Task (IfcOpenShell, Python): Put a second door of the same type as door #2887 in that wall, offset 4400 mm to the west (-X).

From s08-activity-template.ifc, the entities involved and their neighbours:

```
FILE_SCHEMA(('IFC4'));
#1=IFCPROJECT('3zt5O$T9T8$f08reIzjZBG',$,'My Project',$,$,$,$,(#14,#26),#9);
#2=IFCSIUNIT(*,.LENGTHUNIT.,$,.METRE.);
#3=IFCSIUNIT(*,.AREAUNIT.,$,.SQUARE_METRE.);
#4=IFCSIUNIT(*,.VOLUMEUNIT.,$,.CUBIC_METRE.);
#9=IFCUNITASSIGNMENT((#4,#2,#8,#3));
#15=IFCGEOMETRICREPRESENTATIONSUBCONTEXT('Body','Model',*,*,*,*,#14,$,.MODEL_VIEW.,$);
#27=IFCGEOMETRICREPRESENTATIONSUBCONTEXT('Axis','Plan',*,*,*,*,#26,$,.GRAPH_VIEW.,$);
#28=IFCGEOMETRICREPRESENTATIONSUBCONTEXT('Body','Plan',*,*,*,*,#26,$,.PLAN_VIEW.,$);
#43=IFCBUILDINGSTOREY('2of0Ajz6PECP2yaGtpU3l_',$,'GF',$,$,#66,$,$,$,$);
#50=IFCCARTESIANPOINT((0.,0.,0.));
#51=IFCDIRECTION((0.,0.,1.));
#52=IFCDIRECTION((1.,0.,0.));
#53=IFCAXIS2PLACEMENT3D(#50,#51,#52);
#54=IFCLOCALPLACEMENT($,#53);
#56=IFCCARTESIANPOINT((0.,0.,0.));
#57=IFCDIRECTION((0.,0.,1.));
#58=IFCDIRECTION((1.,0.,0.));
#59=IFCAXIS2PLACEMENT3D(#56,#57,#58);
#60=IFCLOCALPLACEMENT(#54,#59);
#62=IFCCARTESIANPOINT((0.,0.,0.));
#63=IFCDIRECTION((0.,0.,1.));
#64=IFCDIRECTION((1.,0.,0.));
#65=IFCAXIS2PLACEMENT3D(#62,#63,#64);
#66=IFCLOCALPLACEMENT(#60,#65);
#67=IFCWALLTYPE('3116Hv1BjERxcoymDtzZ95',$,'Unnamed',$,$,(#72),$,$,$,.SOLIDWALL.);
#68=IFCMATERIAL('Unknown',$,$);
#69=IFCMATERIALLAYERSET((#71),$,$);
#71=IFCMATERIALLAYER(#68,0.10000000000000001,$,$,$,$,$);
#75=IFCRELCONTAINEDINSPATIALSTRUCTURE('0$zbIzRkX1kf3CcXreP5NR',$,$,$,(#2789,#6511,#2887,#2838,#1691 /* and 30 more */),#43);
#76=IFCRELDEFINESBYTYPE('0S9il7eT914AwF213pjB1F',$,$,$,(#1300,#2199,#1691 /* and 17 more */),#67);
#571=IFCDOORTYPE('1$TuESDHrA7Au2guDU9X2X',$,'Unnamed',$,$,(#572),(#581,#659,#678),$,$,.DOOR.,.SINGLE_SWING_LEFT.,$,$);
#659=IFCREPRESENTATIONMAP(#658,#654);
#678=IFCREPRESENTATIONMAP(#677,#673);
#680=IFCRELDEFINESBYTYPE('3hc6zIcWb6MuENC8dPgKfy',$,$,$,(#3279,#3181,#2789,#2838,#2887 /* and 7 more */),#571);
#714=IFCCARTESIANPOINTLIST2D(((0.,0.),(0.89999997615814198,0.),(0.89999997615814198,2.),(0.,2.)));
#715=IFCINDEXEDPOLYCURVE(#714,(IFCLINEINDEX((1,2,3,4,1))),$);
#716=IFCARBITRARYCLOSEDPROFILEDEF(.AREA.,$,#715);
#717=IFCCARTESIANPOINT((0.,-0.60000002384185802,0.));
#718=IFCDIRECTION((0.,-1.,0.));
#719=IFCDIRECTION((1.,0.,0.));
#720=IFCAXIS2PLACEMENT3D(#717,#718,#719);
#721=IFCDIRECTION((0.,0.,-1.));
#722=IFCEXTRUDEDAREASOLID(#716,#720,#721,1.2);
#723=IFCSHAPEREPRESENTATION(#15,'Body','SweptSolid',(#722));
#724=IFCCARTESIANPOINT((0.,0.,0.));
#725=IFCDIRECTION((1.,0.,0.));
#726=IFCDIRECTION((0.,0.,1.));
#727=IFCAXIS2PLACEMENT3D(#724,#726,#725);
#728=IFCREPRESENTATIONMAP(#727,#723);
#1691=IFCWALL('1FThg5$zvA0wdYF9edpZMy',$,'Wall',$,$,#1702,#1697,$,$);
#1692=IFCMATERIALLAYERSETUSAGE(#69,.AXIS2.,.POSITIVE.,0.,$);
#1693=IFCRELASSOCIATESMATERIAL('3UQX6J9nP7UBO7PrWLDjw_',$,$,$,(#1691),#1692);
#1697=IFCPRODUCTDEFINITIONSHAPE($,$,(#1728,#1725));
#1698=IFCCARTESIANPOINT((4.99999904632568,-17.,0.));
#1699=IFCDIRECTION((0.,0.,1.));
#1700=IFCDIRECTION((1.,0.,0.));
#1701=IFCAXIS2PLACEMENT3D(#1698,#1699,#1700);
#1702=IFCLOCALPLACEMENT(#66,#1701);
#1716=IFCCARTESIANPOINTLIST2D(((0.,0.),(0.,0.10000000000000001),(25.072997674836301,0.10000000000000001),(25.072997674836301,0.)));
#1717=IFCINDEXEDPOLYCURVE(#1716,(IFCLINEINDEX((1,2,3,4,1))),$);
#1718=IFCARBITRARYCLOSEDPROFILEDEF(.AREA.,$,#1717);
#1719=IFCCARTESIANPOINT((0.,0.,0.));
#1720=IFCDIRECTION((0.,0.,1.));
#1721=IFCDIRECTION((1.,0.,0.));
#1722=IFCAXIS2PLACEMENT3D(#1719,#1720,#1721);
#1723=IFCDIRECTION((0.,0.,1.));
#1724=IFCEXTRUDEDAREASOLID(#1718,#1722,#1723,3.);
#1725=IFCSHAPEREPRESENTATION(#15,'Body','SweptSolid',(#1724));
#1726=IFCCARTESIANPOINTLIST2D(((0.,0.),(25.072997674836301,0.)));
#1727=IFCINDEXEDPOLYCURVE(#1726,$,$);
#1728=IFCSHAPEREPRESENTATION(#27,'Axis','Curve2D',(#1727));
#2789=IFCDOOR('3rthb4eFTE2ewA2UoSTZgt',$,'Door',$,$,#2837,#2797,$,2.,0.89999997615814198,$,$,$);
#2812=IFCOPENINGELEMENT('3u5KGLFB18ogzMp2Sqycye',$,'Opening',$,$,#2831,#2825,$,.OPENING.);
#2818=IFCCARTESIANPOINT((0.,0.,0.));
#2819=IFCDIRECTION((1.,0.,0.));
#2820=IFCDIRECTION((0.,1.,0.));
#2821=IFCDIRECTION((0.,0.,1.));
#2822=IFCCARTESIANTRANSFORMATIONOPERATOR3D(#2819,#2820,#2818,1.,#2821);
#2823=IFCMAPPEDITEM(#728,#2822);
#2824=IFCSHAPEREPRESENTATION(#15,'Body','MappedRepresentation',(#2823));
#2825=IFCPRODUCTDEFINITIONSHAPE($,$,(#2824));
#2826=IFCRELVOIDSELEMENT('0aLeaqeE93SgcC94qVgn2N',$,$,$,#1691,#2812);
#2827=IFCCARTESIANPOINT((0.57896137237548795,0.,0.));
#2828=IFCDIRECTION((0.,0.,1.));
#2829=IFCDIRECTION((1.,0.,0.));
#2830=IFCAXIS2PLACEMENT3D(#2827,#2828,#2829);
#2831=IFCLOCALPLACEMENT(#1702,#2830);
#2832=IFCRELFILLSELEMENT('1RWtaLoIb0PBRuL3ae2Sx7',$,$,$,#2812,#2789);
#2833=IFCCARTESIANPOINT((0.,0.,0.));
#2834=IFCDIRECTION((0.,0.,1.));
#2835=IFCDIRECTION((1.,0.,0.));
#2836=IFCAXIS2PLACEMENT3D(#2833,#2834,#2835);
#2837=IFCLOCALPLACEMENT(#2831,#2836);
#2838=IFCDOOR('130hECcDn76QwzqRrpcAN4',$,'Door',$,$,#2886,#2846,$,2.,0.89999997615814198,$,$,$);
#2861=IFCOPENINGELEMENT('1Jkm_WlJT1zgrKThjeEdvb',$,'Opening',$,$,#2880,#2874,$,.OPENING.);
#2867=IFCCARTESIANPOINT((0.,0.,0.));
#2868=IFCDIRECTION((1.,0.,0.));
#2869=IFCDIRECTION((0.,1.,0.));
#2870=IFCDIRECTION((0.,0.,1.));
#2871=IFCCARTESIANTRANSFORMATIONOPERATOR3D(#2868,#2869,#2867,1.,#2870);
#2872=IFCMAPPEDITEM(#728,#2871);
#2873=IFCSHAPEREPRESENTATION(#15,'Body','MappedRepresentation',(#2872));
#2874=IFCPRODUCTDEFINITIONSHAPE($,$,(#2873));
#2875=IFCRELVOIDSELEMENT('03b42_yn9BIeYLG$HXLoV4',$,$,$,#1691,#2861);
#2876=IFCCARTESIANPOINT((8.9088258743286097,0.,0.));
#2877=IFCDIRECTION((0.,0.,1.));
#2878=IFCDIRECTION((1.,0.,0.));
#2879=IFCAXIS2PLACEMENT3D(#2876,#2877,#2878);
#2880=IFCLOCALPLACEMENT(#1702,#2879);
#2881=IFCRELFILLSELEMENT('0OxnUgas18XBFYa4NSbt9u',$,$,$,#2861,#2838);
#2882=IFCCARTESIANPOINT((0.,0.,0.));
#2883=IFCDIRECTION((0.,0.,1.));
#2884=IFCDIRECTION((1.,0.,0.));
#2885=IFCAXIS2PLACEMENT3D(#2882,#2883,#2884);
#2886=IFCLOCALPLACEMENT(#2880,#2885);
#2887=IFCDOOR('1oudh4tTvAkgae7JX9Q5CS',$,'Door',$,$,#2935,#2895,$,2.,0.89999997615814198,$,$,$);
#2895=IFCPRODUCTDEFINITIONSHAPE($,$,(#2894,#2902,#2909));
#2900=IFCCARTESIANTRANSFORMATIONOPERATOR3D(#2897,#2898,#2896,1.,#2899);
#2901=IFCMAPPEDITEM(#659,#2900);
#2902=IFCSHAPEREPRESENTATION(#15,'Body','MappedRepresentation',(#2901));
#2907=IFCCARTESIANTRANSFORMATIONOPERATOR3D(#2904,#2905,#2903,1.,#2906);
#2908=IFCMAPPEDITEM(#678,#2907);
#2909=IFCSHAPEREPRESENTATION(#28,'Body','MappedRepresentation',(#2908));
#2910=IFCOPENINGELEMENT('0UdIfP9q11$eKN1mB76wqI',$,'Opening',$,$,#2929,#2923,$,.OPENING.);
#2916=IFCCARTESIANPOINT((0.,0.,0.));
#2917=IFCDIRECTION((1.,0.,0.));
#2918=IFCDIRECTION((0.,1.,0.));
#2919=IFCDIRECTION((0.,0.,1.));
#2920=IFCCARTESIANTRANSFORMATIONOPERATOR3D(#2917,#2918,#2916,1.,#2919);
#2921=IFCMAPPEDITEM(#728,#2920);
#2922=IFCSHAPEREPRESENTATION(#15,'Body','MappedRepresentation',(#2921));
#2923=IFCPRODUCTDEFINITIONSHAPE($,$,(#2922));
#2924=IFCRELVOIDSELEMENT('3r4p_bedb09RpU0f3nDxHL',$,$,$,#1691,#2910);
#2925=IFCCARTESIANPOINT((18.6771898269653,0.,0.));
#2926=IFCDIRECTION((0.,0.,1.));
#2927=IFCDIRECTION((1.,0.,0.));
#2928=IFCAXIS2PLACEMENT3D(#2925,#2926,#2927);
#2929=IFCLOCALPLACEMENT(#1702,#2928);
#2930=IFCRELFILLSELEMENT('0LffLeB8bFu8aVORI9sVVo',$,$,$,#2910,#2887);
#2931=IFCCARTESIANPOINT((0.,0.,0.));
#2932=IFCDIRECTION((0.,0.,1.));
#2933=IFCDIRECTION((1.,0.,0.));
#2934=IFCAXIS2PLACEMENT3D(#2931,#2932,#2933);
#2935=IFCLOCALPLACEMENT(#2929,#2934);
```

```python
import ifcopenshell
import ifcopenshell.api.feature
import ifcopenshell.api.geometry
import ifcopenshell.api.root
import ifcopenshell.geom
import ifcopenshell.util.element
import ifcopenshell.util.placement
import ifcopenshell.util.shape

model = ifcopenshell.open("s08-activity-template.ifc")
settings = ifcopenshell.geom.settings()


def volume(element):
    """Net volume in cubic metres, openings subtracted."""
    shape = ifcopenshell.geom.create_shape(settings, element)
    return ifcopenshell.util.shape.get_volume(shape.geometry)


door = model.by_id(2887)
opening = door.FillsVoids[0].RelatingOpeningElement
wall = opening.VoidsElements[0].RelatingBuildingElement
before = volume(wall)
shift = ifcopenshell.util.placement.get_local_placement(wall.ObjectPlacement)[:3, 0] * -4.4

# copy_class copies the void relationship, type, container and properties, but no geometry.
new_opening = ifcopenshell.api.root.copy_class(model, product=opening)
new_opening.Representation = ifcopenshell.util.element.copy_deep(
    model, opening.Representation, exclude=["IfcGeometricRepresentationContext", "IfcRepresentationMap"]
)
new_door = ifcopenshell.api.root.copy_class(model, product=door)
new_door.Representation = ifcopenshell.util.element.copy_deep(
    model, door.Representation, exclude=["IfcGeometricRepresentationContext", "IfcRepresentationMap"]
)
ifcopenshell.api.feature.add_filling(model, opening=new_opening, element=new_door)

for old, new in ((opening, new_opening), (door, new_door)):
    matrix = ifcopenshell.util.placement.get_local_placement(old.ObjectPlacement)
    matrix[:3, 3] += shift
    ifcopenshell.api.geometry.edit_object_placement(model, product=new, matrix=matrix, is_si=False)

after = volume(wall)

print(f"wall volume {before:.3f} -> {after:.3f} m3")

model.write("s08-activity-template_v2.ifc")
```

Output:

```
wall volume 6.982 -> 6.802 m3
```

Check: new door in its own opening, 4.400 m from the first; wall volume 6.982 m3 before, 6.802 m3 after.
